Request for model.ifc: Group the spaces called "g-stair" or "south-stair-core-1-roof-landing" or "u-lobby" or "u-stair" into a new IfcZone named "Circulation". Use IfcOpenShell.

First a look at what the model holds.

```python
import ifcopenshell

model = ifcopenshell.open("model.ifc")
print(model.schema)
seen = {}
for space in model.by_type("IfcSpace"):
    seen[space.LongName] = seen.get(space.LongName, 0) + 1
for name, count in sorted(seen.items(), key=str):
    print(count, "x", name)
print("zones:", [z.Name for z in model.by_type("IfcZone")][:20])
```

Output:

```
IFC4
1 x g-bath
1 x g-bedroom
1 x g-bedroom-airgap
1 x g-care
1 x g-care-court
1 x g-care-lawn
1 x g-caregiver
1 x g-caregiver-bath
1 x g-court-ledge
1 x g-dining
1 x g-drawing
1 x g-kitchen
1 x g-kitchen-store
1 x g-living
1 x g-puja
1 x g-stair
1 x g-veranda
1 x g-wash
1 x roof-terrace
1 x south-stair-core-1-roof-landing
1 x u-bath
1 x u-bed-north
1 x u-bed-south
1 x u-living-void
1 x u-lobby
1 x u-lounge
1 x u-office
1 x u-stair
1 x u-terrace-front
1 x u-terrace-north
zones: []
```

```python
import ifcopenshell
import ifcopenshell.api.group
import ifcopenshell.api.root

model = ifcopenshell.open("model.ifc")

names = {"g-stair", "south-stair-core-1-roof-landing", "u-lobby", "u-stair"}
spaces = [s for s in model.by_type("IfcSpace") if s.LongName in names]

zone = ifcopenshell.api.root.create_entity(model, ifc_class="IfcZone", name="Circulation")
ifcopenshell.api.group.assign_group(model, products=spaces, group=zone)
print(len(spaces), "spaces in", zone.Name)

model.write("model_edited.ifc")
```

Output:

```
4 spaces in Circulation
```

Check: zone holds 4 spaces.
